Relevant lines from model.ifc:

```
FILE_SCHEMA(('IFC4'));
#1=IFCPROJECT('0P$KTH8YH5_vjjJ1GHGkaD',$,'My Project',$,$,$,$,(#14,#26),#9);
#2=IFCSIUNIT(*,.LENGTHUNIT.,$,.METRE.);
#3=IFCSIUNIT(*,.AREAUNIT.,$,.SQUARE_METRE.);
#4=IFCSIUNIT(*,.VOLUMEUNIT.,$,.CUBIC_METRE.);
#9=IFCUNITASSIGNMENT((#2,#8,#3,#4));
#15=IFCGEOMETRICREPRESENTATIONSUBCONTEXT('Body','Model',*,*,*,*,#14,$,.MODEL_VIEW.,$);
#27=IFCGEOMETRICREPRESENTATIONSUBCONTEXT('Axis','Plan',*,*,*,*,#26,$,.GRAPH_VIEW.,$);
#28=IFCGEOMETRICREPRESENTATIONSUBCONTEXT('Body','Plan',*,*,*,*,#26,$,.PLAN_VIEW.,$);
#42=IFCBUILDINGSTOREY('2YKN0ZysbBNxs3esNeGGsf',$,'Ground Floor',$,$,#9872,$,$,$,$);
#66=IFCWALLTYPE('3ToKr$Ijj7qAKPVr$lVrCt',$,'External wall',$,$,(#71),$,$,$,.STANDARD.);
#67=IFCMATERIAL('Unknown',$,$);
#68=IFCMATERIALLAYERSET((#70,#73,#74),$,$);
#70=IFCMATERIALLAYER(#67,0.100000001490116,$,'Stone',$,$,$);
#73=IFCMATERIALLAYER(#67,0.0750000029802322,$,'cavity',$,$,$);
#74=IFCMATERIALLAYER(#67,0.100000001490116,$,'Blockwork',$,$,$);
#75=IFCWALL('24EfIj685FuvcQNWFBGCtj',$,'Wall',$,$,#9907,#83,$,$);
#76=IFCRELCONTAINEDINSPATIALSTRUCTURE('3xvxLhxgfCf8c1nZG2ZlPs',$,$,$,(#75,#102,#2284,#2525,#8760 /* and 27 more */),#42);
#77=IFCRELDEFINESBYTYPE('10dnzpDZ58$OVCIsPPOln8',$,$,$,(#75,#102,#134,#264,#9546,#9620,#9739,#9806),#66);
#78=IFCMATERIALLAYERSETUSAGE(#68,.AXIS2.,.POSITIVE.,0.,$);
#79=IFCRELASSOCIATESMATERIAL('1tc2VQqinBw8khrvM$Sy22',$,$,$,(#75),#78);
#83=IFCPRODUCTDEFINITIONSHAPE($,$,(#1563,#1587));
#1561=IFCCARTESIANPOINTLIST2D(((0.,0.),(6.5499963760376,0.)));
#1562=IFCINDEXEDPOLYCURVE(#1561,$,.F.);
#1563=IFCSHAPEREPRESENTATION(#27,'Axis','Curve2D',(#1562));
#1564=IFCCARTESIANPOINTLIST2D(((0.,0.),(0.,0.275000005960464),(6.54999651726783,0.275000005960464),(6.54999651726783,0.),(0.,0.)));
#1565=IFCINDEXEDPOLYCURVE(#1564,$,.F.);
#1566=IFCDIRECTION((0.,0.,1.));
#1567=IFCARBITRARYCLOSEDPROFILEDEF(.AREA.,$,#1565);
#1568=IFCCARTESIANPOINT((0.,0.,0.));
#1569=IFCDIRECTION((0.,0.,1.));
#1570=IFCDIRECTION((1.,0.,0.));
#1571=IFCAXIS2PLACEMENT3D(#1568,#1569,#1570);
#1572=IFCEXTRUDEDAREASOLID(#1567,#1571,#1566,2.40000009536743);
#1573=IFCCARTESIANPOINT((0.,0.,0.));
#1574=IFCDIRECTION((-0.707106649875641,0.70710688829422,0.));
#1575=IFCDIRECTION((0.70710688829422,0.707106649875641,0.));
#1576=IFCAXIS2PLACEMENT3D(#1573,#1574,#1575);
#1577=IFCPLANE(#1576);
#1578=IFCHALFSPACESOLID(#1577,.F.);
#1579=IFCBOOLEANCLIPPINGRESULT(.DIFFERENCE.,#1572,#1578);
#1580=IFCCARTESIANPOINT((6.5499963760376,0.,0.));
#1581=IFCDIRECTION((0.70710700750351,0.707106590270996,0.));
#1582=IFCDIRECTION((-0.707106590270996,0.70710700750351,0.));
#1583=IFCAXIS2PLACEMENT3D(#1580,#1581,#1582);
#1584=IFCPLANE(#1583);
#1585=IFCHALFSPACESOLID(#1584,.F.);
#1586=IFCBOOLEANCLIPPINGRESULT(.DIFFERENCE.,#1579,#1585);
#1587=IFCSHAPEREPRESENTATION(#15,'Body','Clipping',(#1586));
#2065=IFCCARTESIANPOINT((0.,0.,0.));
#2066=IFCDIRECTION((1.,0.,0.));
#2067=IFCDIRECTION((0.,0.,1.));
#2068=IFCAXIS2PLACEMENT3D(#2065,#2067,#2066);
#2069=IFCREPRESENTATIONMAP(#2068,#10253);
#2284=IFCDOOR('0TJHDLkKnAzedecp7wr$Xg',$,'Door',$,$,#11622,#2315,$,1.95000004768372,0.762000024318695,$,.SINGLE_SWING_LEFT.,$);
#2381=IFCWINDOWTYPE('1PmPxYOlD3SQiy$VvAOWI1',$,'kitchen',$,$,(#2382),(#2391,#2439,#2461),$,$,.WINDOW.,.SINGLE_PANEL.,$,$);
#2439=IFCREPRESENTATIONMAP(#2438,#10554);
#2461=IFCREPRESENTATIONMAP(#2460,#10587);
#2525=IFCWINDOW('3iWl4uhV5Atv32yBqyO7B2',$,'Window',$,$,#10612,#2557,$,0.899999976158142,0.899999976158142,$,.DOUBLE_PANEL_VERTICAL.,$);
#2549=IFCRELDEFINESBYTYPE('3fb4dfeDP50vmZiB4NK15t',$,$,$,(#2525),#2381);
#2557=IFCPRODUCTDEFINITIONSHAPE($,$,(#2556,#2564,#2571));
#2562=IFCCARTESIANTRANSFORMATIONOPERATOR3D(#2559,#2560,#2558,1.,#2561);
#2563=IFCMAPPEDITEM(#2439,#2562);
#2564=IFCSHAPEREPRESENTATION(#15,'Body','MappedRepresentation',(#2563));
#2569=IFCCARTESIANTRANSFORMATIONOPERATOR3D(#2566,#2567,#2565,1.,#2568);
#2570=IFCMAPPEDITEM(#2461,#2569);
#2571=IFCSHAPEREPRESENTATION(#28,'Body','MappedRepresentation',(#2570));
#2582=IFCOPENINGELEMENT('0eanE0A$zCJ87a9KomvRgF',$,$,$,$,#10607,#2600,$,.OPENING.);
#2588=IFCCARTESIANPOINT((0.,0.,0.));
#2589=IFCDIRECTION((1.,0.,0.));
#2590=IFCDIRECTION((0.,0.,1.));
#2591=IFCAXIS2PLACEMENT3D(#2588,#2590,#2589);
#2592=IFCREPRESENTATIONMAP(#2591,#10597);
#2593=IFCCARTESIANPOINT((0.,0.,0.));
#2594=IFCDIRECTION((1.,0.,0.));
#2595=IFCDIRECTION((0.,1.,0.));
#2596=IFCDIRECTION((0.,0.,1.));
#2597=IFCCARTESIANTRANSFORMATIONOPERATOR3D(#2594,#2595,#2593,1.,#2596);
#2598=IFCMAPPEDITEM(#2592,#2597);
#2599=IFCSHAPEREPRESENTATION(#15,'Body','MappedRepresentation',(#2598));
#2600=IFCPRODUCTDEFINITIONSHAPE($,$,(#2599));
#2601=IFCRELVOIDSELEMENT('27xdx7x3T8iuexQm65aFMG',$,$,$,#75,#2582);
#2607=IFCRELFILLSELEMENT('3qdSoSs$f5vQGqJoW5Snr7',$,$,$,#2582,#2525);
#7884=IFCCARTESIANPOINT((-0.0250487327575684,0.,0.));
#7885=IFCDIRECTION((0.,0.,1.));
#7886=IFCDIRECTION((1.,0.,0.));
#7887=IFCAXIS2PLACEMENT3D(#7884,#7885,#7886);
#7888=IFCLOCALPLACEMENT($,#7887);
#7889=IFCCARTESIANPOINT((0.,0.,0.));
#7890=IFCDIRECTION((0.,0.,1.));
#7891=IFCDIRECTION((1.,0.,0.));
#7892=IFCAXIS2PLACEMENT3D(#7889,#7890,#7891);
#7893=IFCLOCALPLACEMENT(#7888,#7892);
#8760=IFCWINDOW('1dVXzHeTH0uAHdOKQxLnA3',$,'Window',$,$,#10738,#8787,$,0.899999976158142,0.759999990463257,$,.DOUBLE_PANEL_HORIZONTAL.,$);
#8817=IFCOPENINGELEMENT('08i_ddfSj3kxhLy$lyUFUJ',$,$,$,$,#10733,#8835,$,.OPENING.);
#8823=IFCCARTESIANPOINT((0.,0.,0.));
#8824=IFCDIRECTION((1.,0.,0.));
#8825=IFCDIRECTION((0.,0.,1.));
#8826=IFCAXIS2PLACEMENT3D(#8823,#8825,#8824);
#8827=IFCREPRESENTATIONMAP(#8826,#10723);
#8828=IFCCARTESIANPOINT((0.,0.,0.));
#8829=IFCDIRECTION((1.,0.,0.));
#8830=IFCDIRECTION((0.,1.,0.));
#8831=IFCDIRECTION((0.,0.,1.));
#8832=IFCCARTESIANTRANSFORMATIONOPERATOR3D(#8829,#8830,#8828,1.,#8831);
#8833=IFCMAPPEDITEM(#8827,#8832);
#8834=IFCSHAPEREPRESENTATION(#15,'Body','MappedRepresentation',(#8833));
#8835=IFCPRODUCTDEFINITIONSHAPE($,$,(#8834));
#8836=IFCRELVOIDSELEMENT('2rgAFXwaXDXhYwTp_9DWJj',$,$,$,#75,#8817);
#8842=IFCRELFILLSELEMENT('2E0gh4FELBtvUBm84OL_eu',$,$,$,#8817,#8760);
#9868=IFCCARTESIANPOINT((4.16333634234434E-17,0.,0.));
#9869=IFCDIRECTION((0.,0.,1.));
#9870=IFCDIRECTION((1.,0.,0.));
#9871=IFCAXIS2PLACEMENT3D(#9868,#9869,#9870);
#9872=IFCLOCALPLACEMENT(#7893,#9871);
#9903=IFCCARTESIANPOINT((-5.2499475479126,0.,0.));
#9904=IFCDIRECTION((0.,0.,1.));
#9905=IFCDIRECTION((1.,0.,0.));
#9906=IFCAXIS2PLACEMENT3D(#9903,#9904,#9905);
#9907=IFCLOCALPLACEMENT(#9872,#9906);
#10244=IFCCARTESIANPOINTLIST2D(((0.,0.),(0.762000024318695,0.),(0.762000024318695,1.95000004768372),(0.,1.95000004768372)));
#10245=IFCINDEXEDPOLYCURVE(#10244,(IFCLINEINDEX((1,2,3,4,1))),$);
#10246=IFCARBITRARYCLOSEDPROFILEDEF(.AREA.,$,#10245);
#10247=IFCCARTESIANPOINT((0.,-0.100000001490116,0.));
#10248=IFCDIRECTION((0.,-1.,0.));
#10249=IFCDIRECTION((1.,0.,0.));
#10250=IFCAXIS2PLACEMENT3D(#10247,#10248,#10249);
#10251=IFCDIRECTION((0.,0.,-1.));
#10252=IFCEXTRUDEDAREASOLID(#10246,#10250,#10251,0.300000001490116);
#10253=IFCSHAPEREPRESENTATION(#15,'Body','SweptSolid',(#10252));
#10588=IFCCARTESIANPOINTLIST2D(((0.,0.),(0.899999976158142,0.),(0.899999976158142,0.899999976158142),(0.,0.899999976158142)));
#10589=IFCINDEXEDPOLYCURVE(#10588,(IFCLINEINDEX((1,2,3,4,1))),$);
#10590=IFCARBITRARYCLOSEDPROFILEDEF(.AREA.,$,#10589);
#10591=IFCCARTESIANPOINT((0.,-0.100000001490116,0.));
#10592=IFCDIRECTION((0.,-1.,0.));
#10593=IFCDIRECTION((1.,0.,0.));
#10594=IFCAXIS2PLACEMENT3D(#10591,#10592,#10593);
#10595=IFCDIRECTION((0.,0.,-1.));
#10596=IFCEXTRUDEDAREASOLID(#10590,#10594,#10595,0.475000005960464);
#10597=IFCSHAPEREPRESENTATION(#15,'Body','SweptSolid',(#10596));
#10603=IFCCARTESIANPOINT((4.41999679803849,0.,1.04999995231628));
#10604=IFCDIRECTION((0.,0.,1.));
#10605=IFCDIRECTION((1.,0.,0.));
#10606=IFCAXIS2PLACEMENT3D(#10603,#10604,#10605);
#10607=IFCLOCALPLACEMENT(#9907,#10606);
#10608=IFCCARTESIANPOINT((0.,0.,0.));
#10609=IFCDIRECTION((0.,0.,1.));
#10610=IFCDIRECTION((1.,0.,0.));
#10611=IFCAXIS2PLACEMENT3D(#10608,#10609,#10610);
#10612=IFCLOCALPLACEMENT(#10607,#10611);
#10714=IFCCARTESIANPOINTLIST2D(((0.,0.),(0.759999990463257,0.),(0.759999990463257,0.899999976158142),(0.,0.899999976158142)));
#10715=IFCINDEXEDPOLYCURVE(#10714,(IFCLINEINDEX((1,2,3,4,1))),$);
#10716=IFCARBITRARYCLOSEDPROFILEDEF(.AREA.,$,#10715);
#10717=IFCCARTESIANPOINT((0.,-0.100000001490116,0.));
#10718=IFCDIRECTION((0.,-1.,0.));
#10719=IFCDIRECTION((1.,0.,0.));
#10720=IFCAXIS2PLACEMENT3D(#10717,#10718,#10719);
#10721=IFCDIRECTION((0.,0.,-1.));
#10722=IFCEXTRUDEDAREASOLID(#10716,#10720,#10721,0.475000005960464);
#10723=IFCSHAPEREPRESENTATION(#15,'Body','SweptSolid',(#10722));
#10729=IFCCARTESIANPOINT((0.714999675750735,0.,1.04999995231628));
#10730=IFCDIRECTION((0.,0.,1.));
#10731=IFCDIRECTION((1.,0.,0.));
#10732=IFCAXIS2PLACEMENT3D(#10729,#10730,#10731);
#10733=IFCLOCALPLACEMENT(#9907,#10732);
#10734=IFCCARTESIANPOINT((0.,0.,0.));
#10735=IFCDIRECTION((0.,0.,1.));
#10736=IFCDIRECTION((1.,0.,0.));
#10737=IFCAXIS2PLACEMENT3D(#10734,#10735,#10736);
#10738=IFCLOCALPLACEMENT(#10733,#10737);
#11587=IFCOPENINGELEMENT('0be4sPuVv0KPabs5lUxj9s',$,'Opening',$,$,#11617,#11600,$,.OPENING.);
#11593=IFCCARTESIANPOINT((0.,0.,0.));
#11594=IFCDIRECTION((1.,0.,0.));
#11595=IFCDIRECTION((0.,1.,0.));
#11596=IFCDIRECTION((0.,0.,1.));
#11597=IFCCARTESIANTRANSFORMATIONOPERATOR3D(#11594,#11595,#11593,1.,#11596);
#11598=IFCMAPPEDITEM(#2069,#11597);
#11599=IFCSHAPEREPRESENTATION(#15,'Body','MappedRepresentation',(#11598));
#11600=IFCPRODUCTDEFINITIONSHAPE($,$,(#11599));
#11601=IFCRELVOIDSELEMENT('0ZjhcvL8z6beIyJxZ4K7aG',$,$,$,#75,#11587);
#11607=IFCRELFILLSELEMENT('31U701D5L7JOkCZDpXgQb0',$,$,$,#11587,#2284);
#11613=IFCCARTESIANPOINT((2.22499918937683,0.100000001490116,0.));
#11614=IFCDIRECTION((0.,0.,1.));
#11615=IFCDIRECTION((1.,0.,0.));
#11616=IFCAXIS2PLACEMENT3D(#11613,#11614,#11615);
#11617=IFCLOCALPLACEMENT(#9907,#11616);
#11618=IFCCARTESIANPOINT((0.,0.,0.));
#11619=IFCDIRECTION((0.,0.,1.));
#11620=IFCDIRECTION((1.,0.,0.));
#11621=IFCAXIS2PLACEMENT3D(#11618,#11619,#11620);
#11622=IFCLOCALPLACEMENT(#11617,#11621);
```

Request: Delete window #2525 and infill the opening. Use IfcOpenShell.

```python
import ifcopenshell
import ifcopenshell.api.feature
import ifcopenshell.api.root
import ifcopenshell.geom
import ifcopenshell.util.shape

model = ifcopenshell.open("model.ifc")
settings = ifcopenshell.geom.settings()


def volume(element):
    """Net volume in cubic metres, openings subtracted."""
    shape = ifcopenshell.geom.create_shape(settings, element)
    return ifcopenshell.util.shape.get_volume(shape.geometry)


window = model.by_guid("3iWl4uhV5Atv32yBqyO7B2")
opening = window.FillsVoids[0].RelatingOpeningElement
wall = opening.VoidsElements[0].RelatingBuildingElement
before = volume(wall)

ifcopenshell.api.root.remove_product(model, product=window)
ifcopenshell.api.feature.remove_feature(model, feature=opening)

after = volume(wall)

print(f"wall volume {before:.3f} -> {after:.3f} m3")

model.write("model-out.ifc")
```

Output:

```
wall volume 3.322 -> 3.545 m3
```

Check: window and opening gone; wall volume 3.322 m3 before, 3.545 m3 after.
